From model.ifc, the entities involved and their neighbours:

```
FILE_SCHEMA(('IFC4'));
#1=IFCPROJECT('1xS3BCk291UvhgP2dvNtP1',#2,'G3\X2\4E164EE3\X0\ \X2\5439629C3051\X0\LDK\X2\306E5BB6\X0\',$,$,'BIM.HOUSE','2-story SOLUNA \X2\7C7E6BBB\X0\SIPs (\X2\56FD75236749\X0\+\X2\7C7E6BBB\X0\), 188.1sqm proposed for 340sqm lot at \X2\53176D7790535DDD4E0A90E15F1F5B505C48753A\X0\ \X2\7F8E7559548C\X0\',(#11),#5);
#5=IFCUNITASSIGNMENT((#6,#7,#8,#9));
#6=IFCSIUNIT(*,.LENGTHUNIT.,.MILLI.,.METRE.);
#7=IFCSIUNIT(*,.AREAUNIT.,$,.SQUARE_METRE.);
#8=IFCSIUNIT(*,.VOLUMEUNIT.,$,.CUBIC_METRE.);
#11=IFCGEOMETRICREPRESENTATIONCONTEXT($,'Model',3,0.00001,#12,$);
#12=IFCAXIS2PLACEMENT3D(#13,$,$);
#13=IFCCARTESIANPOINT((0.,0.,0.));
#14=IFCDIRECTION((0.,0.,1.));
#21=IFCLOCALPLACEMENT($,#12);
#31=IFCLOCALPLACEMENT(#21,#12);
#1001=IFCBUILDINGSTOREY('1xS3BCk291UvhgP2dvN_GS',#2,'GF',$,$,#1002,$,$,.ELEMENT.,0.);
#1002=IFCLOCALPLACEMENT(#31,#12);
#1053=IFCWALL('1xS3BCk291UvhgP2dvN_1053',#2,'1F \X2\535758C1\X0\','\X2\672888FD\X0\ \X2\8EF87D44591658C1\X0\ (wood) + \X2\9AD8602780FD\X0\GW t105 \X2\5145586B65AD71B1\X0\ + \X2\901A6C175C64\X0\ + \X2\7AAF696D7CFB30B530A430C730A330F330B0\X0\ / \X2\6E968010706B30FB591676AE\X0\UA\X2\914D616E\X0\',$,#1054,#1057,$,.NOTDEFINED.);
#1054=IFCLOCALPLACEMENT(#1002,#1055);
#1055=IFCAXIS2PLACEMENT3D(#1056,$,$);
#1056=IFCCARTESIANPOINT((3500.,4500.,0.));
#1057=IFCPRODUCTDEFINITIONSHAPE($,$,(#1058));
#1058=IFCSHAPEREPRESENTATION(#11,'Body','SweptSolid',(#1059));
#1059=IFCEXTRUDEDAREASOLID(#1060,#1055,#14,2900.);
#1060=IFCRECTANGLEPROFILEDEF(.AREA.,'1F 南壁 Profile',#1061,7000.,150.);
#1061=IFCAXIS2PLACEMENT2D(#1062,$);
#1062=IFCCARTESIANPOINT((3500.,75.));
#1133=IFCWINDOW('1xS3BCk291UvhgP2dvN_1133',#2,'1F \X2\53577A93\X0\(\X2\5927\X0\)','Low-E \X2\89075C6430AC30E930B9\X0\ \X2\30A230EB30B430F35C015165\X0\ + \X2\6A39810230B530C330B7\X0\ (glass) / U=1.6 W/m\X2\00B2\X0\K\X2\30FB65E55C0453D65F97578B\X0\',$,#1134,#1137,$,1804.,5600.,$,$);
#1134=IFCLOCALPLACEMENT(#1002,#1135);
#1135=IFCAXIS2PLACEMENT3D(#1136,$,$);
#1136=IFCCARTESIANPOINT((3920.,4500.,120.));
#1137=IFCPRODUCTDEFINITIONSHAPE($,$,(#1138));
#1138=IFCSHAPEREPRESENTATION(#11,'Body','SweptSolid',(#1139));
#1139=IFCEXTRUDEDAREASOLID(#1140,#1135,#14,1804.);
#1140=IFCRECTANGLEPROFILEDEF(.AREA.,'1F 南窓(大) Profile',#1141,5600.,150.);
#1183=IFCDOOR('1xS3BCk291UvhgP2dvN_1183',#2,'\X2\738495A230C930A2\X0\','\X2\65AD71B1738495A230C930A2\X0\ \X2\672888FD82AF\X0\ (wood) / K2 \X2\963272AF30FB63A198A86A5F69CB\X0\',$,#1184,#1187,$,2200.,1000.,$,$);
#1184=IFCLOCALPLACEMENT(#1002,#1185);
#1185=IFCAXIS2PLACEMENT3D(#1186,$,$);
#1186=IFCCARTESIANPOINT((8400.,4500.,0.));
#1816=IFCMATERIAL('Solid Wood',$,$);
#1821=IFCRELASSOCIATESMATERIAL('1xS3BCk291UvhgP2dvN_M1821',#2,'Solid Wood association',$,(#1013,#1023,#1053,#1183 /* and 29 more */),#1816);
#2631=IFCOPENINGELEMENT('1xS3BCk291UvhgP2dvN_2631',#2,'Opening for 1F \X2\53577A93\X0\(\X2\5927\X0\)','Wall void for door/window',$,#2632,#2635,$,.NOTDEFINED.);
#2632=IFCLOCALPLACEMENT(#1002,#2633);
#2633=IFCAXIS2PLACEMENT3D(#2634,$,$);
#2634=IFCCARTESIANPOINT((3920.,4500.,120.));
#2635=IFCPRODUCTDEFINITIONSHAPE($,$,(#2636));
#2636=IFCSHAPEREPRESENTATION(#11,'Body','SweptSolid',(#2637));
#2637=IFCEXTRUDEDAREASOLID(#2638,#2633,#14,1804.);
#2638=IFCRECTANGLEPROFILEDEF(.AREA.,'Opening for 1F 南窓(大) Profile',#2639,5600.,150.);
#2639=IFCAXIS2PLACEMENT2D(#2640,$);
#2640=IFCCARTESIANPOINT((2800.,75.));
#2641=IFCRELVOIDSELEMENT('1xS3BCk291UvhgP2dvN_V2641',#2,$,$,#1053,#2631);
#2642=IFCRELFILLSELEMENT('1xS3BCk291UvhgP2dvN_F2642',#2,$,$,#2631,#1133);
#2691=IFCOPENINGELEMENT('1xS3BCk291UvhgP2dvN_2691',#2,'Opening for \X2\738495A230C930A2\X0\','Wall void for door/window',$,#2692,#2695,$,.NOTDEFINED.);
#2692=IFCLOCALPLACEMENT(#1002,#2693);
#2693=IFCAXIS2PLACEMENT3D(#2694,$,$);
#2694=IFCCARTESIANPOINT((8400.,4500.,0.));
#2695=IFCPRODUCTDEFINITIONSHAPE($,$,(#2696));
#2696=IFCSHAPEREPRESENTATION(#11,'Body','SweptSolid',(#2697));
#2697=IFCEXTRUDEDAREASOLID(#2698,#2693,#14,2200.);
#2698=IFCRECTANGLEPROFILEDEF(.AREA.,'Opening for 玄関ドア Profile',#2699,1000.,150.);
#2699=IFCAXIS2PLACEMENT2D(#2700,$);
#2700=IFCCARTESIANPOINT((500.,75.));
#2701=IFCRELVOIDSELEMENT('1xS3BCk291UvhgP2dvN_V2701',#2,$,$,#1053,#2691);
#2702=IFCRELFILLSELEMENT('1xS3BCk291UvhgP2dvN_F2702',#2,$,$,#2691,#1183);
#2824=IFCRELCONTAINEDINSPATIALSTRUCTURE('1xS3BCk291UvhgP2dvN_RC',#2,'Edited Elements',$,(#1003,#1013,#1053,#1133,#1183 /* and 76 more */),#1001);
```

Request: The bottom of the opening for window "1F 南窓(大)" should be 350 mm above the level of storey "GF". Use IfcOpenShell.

```python
import numpy as np
import ifcopenshell
import ifcopenshell.api.geometry
import ifcopenshell.geom
import ifcopenshell.util.element
import ifcopenshell.util.placement
import ifcopenshell.util.shape
import ifcopenshell.util.unit

model = ifcopenshell.open("model.ifc")
unit_scale = ifcopenshell.util.unit.calculate_unit_scale(model)

window = model.by_guid("1xS3BCk291UvhgP2dvN_1133")
opening = window.FillsVoids[0].RelatingOpeningElement
storey = ifcopenshell.util.element.get_container(window, ifc_class="IfcBuildingStorey")
level = ifcopenshell.util.placement.get_local_placement(storey.ObjectPlacement)[2, 3]

# The opening's origin need not be at the sill, so measure its lowest point.
shape = ifcopenshell.geom.create_shape(ifcopenshell.geom.settings(), opening)
bottom = ifcopenshell.util.shape.get_shape_bottom_elevation(shape, shape.geometry) / unit_scale
dz = level + 350.0 - bottom

shift = np.array([0.0, 0.0, dz])
# The window is not placed relative to its opening, so move both.
for product in (opening, window):
    matrix = ifcopenshell.util.placement.get_local_placement(product.ObjectPlacement)
    matrix[:3, 3] += shift
    ifcopenshell.api.geometry.edit_object_placement(model, product=product, matrix=matrix, is_si=False)

print(f"moved by {dz * unit_scale:+.3f} m")

model.write("model-out.ifc")
```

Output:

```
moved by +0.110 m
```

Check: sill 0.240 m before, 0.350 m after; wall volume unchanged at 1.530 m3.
